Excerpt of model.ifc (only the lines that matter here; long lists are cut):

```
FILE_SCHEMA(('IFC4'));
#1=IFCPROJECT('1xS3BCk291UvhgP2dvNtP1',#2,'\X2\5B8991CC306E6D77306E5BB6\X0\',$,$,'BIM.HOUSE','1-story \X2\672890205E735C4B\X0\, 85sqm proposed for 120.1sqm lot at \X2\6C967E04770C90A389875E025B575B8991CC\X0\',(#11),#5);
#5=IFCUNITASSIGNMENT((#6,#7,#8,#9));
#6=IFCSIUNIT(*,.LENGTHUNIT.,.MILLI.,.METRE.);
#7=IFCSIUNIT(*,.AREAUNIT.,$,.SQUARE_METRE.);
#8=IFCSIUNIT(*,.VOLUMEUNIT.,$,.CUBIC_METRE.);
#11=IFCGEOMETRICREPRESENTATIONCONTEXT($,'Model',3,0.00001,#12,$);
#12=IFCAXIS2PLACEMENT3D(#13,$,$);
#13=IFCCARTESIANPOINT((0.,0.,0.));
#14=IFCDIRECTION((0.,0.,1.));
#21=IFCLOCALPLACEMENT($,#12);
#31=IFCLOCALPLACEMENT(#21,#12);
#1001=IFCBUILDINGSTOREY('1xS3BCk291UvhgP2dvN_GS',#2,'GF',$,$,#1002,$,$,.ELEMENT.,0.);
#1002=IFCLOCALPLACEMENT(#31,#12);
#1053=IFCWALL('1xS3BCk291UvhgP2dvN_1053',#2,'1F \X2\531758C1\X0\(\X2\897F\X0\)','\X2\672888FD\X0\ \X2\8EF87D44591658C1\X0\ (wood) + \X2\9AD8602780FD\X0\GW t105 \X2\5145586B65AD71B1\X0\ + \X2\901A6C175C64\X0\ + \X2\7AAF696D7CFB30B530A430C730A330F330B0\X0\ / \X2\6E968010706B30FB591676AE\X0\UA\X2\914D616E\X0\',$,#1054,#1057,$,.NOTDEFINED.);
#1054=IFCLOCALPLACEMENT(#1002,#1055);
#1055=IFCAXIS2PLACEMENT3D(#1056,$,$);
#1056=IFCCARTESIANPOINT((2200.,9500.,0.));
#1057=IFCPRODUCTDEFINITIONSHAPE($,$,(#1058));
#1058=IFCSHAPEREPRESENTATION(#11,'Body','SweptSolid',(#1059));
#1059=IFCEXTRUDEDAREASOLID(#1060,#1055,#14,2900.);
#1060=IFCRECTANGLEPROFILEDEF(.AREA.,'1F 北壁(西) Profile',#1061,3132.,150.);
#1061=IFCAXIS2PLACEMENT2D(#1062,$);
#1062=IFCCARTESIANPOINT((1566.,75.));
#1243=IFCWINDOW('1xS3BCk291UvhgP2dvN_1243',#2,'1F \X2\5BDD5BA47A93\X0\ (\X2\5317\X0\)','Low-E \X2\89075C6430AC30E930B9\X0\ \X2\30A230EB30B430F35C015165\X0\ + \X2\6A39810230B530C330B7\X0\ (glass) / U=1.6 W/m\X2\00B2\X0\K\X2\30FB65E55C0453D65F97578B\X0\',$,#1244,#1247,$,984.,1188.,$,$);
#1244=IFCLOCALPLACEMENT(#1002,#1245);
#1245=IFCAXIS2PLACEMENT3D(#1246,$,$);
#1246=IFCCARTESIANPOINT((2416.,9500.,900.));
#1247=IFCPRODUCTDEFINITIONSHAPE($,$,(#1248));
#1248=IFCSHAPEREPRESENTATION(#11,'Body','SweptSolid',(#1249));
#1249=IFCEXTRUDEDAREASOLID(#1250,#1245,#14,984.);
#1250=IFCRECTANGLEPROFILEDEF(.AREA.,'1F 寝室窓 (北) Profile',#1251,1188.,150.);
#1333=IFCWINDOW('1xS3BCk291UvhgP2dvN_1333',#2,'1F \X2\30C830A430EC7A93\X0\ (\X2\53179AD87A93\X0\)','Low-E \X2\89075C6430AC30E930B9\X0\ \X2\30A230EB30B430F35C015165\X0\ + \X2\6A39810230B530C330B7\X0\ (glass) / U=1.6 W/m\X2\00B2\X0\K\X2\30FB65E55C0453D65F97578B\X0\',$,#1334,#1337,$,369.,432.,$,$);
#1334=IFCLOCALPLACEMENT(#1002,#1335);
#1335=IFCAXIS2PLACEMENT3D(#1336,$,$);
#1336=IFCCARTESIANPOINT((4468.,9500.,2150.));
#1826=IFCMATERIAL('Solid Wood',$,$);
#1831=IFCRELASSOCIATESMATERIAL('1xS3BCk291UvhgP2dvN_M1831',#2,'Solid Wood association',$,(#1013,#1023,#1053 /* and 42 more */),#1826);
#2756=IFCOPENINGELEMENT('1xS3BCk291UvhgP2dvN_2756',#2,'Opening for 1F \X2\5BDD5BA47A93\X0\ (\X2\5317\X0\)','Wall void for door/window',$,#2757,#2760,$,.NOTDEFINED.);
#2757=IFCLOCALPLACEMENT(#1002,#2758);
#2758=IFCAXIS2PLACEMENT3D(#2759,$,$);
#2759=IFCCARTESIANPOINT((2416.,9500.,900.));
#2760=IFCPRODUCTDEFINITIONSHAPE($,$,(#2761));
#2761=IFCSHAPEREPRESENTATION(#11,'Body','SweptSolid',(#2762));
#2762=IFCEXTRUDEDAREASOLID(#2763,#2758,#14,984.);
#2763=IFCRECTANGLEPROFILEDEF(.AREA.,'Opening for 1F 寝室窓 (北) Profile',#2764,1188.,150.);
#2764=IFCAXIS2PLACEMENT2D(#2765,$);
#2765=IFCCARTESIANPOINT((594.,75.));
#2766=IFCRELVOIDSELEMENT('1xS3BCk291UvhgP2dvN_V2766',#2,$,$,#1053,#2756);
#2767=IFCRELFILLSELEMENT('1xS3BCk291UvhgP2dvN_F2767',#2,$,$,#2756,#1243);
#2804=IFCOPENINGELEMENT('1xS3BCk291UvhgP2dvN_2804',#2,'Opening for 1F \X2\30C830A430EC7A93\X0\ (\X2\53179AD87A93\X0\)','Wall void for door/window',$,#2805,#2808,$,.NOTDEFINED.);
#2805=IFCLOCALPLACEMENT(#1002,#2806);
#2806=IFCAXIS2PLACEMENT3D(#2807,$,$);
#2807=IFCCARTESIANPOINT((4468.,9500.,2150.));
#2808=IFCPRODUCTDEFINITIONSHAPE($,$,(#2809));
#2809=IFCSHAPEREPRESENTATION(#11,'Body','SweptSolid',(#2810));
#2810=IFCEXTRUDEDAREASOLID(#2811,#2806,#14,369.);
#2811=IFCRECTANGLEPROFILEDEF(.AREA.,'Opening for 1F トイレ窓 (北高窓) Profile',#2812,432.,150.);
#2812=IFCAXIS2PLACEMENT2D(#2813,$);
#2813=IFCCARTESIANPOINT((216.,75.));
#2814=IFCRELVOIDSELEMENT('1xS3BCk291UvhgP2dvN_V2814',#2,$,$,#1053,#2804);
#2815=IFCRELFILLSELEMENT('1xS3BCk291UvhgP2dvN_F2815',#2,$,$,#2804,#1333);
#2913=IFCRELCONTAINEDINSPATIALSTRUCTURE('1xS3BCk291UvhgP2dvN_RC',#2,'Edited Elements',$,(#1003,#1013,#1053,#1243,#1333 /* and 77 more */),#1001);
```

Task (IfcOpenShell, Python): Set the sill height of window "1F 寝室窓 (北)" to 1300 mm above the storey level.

```python
import numpy as np
import ifcopenshell
import ifcopenshell.api.geometry
import ifcopenshell.geom
import ifcopenshell.util.element
import ifcopenshell.util.placement
import ifcopenshell.util.shape
import ifcopenshell.util.unit

model = ifcopenshell.open("model.ifc")
unit_scale = ifcopenshell.util.unit.calculate_unit_scale(model)

window = model.by_guid("1xS3BCk291UvhgP2dvN_1243")
opening = window.FillsVoids[0].RelatingOpeningElement
storey = ifcopenshell.util.element.get_container(window, ifc_class="IfcBuildingStorey")
level = ifcopenshell.util.placement.get_local_placement(storey.ObjectPlacement)[2, 3]

# The opening's origin need not be at the sill, so measure its lowest point.
shape = ifcopenshell.geom.create_shape(ifcopenshell.geom.settings(), opening)
bottom = ifcopenshell.util.shape.get_shape_bottom_elevation(shape, shape.geometry) / unit_scale
dz = level + 1.3 / unit_scale - bottom

shift = np.array([0.0, 0.0, dz])
# The window is not placed relative to its opening, so move both.
for product in (opening, window):
    matrix = ifcopenshell.util.placement.get_local_placement(product.ObjectPlacement)
    matrix[:3, 3] += shift
    ifcopenshell.api.geometry.edit_object_placement(model, product=product, matrix=matrix, is_si=False)

print(f"moved by {dz * unit_scale:+.3f} m")

model.write("model_updated.ifc")
```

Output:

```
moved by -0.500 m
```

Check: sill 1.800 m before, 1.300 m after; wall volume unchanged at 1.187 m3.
